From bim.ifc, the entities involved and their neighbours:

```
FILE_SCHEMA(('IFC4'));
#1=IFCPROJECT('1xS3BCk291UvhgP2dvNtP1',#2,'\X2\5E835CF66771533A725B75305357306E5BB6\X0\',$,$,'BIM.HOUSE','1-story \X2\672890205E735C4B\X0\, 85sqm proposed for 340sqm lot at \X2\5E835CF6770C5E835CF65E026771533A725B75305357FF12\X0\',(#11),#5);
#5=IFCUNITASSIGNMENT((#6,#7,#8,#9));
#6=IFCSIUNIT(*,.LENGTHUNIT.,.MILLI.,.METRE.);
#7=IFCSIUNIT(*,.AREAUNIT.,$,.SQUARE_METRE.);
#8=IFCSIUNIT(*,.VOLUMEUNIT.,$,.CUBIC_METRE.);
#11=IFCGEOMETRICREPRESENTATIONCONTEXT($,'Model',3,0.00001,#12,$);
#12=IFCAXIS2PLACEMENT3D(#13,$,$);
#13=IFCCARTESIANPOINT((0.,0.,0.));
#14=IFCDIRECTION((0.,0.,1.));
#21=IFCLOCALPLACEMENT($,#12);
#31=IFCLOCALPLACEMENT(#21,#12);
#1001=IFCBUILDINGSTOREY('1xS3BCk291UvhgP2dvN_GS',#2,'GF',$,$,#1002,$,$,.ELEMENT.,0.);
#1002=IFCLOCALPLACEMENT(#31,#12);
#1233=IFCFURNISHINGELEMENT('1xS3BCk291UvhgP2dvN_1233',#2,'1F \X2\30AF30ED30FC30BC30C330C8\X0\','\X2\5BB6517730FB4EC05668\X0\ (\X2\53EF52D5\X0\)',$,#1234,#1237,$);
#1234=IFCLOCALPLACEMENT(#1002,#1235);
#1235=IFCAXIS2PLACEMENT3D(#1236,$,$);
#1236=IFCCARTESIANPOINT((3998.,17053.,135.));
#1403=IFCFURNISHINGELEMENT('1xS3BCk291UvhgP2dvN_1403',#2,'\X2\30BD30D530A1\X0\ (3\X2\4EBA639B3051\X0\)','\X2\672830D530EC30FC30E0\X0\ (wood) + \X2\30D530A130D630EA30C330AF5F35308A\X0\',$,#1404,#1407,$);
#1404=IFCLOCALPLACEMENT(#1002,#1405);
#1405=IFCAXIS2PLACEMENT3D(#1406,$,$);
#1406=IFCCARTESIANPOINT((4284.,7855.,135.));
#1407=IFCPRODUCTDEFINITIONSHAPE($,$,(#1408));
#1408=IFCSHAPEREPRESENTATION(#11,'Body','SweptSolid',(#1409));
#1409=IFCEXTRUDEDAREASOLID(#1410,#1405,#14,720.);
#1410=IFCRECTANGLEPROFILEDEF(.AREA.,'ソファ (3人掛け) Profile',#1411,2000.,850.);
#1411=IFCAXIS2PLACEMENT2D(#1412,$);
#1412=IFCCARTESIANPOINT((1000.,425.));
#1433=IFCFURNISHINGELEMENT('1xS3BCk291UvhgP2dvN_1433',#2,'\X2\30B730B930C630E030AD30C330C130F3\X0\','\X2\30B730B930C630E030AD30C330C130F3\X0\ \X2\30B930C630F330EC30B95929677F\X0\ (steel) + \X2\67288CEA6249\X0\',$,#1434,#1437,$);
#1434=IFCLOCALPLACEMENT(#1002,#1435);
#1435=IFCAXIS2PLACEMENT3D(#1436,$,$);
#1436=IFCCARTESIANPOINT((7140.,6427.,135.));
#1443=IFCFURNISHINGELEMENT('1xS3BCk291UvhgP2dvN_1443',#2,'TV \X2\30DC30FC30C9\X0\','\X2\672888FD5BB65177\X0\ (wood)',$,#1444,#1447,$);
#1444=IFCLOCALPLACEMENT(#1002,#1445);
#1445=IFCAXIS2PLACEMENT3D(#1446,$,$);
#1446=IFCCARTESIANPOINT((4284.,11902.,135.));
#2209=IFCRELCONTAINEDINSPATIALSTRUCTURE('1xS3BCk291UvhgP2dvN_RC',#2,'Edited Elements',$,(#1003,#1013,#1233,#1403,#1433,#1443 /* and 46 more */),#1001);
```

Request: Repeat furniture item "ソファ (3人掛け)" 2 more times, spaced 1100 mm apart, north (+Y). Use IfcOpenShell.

```python
import numpy as np
import ifcopenshell
import ifcopenshell.api.geometry
import ifcopenshell.api.root
import ifcopenshell.util.element
import ifcopenshell.util.placement

model = ifcopenshell.open("bim.ifc")


def reuse_history(source, copy):
    """copy_class also copies each property set's owner history, people and application; keep the originals."""
    for rel in copy.IsDefinedBy:
        if rel.is_a("IfcRelDefinesByProperties") and (history := rel.RelatingPropertyDefinition.OwnerHistory):
            rel.RelatingPropertyDefinition.OwnerHistory = source.OwnerHistory
            ifcopenshell.util.element.remove_deep2(model, history)


source = model.by_guid("1xS3BCk291UvhgP2dvN_1403")
base = ifcopenshell.util.placement.get_local_placement(source.ObjectPlacement)
step = np.array([0.0, 1.0, 0.0]) * 1100.0

for i in range(1, 3):
    copy = ifcopenshell.api.root.copy_class(model, product=source)
    copy.Representation = ifcopenshell.util.element.copy_deep(
        model, source.Representation, exclude=["IfcGeometricRepresentationContext", "IfcRepresentationMap"]
    )
    reuse_history(source, copy)
    matrix = base.copy()
    matrix[:3, 3] += i * step
    print("added at", matrix[:3, 3].round(3) + 0.0)
    ifcopenshell.api.geometry.edit_object_placement(model, product=copy, matrix=matrix, is_si=False)

model.write("bim_rev.ifc")
```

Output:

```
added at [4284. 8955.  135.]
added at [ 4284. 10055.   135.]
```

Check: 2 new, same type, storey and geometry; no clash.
